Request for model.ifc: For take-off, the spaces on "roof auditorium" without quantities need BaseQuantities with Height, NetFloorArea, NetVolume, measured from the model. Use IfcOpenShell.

First a look at what the model holds.

```python
import ifcopenshell
import ifcopenshell.util.element
import ifcopenshell.util.unit

model = ifcopenshell.open("model.ifc")
print(model.schema)
for unit_type in ("LENGTHUNIT", "AREAUNIT", "VOLUMEUNIT"):
    print(unit_type, ifcopenshell.util.unit.calculate_unit_scale(model, unit_type))
storey = next(s for s in model.by_type("IfcBuildingStorey") if s.Name == "roof auditorium")
spaces = [e for e in ifcopenshell.util.element.get_decomposition(storey) if e.is_a("IfcSpace")]
for e in sorted(spaces, key=lambda e: e.id()):
    print(e.id(), e.is_a(), e.Name, list(ifcopenshell.util.element.get_psets(e, qtos_only=True)), sep=" | ")
```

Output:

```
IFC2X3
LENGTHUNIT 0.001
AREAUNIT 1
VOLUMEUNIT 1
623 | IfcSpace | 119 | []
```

```python
import ifcopenshell
import ifcopenshell.api.pset
import ifcopenshell.geom
import ifcopenshell.util.element
import ifcopenshell.util.shape
import ifcopenshell.util.unit

model = ifcopenshell.open("model.ifc")
unit_scale = ifcopenshell.util.unit.calculate_unit_scale(model)
area_scale = ifcopenshell.util.unit.calculate_unit_scale(model, "AREAUNIT")
volume_scale = ifcopenshell.util.unit.calculate_unit_scale(model, "VOLUMEUNIT")
settings = ifcopenshell.geom.settings()

storey = next(s for s in model.by_type("IfcBuildingStorey") if s.Name == "roof auditorium")
spaces = [e for e in ifcopenshell.util.element.get_decomposition(storey) if e.is_a("IfcSpace")]

for e in sorted(spaces, key=lambda e: e.id()):
    if ifcopenshell.util.element.get_psets(e, qtos_only=True, should_inherit=False):
        continue
    # Geometry comes back in metres, in the element's own axes.
    shape = ifcopenshell.geom.create_shape(settings, e)
    values = {
        "Height": ifcopenshell.util.shape.get_z(shape.geometry) / unit_scale,
        "NetFloorArea": ifcopenshell.util.shape.get_footprint_area(shape.geometry) / area_scale,
        "NetVolume": ifcopenshell.util.shape.get_volume(shape.geometry) / volume_scale,
    }
    qto = ifcopenshell.api.pset.add_qto(model, product=e, name="BaseQuantities")
    ifcopenshell.api.pset.edit_qto(model, qto=qto, properties=values)
    print(e.id(), {k: round(v, 3) for k, v in values.items()})

model.write("model_updated.ifc")
```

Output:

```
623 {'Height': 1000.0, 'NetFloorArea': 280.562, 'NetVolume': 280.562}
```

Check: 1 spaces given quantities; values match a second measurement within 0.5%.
